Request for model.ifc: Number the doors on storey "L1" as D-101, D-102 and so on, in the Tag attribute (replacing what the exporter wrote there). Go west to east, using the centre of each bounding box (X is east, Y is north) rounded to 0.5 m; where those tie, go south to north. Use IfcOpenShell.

First a look at what the model holds.

```python
import ifcopenshell
import ifcopenshell.util.element
import ifcopenshell.util.placement

model = ifcopenshell.open("model.ifc")
print(model.schema)
storey = next(s for s in model.by_type("IfcBuildingStorey") if s.Name == "L1")
doors = [e for e in ifcopenshell.util.element.get_decomposition(storey) if e.is_a("IfcDoor")]
for e in sorted(doors, key=lambda e: e.id()):
    origin = ifcopenshell.util.placement.get_local_placement(e.ObjectPlacement)[:3, 3]
    print(e.id(), e.Tag, e.Name, origin.round(2) + 0.0, sep=" | ")
```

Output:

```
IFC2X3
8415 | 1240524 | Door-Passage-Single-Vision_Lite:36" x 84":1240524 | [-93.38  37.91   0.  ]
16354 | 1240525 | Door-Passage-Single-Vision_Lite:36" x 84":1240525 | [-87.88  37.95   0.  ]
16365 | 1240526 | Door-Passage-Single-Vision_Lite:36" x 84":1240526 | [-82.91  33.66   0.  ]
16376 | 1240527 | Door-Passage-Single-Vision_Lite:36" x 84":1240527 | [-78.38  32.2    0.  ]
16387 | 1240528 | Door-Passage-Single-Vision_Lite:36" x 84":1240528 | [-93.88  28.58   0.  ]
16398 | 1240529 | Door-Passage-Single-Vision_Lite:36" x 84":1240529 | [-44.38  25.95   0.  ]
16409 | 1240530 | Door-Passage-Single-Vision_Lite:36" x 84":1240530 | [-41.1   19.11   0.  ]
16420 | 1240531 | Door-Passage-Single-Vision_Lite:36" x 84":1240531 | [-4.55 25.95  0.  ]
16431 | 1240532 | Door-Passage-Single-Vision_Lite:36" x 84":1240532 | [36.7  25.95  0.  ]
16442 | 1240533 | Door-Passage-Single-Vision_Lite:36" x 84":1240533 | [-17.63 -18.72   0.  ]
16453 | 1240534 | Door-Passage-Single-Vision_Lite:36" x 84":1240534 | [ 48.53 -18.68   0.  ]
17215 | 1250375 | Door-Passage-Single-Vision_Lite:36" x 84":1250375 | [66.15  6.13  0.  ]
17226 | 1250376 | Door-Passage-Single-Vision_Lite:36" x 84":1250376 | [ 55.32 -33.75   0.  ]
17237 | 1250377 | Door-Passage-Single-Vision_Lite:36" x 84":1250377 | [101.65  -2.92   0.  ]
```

```python
import ifcopenshell
import ifcopenshell.geom
import ifcopenshell.util.element
import ifcopenshell.util.shape

model = ifcopenshell.open("model.ifc")
settings = ifcopenshell.geom.settings()
settings.set("use-world-coords", True)


def centre(element):
    shape = ifcopenshell.geom.create_shape(settings, element)
    return ifcopenshell.util.shape.get_bbox_centroid(shape.geometry)


storey = next(s for s in model.by_type("IfcBuildingStorey") if s.Name == "L1")
doors = [e for e in ifcopenshell.util.element.get_decomposition(storey) if e.is_a("IfcDoor")]

# Insertion points can sit at a corner or the storey origin, so sort by the geometry (in metres).
centres = {e: centre(e) for e in doors}
doors.sort(key=lambda e: (round(centres[e][0] / 0.5), centres[e][1]))

for i, e in enumerate(doors, start=1):
    number = f"D-1{i:02d}"
    e.Tag = number
    print(e.id(), number)

model.write("model_edited.ifc")
```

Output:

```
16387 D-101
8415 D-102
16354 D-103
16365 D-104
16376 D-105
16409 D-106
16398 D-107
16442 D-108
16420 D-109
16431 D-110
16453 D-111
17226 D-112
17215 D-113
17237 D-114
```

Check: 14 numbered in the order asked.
